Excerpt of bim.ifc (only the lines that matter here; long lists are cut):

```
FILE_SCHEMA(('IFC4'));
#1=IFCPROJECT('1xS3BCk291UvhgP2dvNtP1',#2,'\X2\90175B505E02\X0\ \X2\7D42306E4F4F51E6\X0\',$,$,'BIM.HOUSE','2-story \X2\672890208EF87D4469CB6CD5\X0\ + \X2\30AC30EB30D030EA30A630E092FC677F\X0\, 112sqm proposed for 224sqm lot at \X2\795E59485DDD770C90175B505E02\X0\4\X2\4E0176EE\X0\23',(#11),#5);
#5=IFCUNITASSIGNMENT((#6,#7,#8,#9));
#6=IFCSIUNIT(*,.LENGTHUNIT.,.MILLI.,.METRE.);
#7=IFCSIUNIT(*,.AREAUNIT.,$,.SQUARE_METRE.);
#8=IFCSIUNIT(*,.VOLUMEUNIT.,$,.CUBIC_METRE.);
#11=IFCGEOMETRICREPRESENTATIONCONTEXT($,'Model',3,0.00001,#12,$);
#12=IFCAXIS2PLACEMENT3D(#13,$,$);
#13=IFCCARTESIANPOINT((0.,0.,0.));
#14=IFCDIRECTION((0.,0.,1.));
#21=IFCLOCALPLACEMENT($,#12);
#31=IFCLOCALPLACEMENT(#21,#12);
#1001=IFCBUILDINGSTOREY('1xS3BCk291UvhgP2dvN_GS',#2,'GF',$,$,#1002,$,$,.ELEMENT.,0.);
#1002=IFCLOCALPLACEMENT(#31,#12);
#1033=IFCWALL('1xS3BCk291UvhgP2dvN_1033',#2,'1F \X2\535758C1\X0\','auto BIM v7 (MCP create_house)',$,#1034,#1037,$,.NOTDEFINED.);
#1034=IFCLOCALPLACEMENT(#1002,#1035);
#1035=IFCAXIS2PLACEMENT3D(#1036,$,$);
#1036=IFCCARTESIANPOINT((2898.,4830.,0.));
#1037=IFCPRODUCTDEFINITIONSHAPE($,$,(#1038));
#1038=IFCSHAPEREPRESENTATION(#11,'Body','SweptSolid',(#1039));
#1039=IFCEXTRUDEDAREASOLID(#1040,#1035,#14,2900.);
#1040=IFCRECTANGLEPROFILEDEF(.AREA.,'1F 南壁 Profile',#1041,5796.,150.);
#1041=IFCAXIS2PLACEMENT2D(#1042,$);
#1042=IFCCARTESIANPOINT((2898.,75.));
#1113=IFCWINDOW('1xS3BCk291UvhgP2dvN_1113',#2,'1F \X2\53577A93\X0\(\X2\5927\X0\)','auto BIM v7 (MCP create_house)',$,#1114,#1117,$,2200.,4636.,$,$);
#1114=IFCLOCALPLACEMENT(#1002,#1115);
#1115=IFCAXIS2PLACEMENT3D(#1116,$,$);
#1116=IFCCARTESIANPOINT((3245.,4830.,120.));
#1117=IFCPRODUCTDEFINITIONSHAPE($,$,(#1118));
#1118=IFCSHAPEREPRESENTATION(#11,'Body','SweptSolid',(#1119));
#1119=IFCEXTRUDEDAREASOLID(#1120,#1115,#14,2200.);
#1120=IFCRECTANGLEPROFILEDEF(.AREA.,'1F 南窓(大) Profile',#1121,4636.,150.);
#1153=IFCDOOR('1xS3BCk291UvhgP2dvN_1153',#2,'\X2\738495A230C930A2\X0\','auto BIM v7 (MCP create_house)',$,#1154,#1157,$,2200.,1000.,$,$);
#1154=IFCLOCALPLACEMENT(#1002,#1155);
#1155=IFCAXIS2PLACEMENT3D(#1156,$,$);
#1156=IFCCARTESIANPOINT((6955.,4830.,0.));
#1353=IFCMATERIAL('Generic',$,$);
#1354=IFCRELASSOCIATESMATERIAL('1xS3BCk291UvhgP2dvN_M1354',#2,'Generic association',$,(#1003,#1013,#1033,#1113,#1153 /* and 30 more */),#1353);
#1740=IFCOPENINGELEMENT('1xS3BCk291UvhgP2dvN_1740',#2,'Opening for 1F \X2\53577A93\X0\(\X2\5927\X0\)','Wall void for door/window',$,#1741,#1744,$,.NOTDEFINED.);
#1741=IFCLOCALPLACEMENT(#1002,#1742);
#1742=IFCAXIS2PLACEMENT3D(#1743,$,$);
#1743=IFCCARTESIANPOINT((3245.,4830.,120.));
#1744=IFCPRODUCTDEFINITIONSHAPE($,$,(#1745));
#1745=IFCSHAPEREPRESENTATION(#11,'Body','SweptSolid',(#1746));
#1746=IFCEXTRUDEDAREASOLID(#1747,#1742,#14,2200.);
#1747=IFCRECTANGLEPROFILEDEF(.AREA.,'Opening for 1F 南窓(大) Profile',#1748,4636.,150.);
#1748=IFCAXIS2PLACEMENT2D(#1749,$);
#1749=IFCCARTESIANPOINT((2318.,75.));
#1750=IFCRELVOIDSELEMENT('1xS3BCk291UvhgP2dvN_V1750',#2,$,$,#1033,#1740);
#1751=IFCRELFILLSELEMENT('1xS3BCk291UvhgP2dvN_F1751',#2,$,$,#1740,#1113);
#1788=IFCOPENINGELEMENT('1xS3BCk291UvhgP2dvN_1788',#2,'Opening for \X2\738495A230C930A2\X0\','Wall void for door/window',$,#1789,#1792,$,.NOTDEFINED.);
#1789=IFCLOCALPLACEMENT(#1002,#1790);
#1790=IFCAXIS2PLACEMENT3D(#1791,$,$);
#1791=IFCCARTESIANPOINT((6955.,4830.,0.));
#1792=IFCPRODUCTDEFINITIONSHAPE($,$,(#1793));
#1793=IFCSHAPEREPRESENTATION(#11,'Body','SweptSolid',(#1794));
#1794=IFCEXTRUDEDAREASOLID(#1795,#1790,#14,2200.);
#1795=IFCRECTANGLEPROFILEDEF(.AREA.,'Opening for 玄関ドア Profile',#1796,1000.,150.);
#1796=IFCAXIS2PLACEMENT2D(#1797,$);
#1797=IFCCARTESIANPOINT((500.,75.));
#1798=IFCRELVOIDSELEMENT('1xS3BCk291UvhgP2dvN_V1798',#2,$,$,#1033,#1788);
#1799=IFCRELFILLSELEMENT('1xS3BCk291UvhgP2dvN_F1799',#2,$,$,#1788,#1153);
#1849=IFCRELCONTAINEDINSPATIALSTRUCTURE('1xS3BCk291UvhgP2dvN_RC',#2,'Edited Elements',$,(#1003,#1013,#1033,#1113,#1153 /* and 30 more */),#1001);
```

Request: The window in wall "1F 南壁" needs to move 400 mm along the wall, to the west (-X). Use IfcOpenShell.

```python
import ifcopenshell
import ifcopenshell.api.geometry
import ifcopenshell.util.placement
import ifcopenshell.util.unit

model = ifcopenshell.open("bim.ifc")
unit_scale = ifcopenshell.util.unit.calculate_unit_scale(model)

window = model.by_guid("1xS3BCk291UvhgP2dvN_1113")
opening = window.FillsVoids[0].RelatingOpeningElement
wall = opening.VoidsElements[0].RelatingBuildingElement

wall_matrix = ifcopenshell.util.placement.get_local_placement(wall.ObjectPlacement)
shift = wall_matrix[:3, 0] * -0.4 / unit_scale
before = ifcopenshell.util.placement.get_local_placement(window.ObjectPlacement)[:3, 3].copy()

# The window is not placed relative to its opening, so move both.
for product in (opening, window):
    matrix = ifcopenshell.util.placement.get_local_placement(product.ObjectPlacement)
    matrix[:3, 3] += shift
    ifcopenshell.api.geometry.edit_object_placement(model, product=product, matrix=matrix, is_si=False)

after = ifcopenshell.util.placement.get_local_placement(window.ObjectPlacement)[:3, 3]
print("window moved by", (after - before).round(3) + 0.0)

model.write("bim_updated.ifc")
```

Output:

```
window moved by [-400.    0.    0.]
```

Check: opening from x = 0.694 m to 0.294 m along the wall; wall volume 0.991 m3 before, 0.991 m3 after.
